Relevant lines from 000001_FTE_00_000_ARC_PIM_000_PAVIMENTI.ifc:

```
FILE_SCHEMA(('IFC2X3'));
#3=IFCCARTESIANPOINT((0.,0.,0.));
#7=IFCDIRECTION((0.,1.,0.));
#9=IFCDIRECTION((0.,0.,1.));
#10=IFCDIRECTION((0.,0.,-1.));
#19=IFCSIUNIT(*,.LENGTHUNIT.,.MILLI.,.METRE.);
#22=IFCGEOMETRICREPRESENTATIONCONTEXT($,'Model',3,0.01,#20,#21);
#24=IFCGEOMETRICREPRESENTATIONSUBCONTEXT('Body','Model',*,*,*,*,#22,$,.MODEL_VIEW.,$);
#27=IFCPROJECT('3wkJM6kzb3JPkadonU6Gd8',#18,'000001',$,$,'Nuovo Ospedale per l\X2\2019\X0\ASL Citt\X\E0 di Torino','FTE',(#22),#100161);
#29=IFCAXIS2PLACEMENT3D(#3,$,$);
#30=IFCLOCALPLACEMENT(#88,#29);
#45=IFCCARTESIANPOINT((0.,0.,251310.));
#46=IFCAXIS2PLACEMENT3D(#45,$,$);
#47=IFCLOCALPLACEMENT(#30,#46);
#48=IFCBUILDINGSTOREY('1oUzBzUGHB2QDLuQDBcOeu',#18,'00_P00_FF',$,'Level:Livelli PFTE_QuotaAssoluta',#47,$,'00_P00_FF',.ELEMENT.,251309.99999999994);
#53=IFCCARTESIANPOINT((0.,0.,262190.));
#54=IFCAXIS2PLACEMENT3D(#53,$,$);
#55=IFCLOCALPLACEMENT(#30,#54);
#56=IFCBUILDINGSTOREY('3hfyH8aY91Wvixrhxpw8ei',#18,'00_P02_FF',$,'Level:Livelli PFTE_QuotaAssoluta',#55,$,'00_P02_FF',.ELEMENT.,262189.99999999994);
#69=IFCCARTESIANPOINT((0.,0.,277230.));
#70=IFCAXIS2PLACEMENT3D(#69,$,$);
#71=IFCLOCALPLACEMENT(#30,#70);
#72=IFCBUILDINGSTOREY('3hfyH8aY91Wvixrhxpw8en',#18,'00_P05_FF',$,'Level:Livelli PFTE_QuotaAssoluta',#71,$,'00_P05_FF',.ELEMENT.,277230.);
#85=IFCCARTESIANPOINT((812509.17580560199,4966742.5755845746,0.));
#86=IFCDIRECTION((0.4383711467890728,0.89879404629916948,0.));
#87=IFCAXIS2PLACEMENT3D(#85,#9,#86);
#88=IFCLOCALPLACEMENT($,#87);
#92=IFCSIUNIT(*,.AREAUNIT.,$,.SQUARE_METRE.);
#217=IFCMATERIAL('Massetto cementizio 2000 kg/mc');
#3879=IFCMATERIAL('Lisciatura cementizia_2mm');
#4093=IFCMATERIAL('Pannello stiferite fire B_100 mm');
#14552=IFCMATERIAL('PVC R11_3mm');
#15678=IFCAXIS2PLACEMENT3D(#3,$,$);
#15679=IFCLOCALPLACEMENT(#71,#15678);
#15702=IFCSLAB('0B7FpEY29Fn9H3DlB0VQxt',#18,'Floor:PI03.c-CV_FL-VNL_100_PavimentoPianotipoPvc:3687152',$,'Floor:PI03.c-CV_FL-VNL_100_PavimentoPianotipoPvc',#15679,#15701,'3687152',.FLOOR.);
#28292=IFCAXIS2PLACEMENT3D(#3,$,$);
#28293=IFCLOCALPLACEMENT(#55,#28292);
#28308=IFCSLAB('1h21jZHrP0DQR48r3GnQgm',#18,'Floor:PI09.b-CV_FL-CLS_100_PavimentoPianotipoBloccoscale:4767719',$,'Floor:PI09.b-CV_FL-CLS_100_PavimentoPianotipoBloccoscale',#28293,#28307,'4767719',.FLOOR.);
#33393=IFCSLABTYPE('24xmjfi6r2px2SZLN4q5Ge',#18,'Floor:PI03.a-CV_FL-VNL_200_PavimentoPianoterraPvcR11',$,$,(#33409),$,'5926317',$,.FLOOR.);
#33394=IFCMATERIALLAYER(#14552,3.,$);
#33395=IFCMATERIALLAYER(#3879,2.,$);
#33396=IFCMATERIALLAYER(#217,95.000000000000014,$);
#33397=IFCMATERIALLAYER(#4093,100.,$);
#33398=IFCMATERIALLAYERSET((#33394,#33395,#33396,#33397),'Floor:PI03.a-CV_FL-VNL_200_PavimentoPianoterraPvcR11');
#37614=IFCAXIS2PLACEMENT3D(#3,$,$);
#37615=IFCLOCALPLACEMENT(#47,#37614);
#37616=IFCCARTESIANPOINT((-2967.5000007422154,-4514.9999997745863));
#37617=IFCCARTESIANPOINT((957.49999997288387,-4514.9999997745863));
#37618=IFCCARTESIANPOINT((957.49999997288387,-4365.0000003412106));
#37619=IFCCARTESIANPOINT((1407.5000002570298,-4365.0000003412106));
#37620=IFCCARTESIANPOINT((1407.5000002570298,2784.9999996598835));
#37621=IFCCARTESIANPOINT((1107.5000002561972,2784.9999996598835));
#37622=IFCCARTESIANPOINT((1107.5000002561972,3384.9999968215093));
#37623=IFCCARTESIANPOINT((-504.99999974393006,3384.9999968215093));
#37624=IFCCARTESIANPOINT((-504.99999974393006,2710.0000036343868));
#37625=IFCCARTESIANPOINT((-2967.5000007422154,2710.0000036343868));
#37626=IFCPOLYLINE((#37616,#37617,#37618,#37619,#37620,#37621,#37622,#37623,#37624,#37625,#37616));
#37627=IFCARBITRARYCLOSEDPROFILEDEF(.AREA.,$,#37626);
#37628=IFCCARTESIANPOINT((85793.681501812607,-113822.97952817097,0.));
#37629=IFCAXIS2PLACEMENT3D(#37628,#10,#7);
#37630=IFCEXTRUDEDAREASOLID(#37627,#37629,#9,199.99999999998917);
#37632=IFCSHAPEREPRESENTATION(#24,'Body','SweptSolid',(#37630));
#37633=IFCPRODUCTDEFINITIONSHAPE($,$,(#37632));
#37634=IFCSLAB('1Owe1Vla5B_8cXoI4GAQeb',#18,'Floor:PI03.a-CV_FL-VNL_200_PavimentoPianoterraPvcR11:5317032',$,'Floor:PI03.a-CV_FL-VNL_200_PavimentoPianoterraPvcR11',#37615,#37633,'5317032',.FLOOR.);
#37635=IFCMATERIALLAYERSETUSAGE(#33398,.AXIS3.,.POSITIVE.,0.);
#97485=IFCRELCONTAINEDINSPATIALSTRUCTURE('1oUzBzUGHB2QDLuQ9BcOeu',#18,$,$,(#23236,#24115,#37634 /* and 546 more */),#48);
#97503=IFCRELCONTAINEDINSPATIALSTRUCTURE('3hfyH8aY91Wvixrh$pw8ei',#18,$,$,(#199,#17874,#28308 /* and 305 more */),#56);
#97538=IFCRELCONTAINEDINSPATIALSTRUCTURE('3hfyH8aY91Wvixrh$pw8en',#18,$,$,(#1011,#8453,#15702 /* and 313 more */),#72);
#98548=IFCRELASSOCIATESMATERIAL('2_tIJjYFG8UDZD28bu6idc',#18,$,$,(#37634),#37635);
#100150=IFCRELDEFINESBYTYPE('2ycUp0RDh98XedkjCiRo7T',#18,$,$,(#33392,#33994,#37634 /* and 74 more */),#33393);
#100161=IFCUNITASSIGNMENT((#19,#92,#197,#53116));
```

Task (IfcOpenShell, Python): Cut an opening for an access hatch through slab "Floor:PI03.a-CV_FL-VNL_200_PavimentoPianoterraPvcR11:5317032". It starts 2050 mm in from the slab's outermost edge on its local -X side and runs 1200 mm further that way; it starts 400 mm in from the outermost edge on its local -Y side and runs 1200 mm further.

```python
import numpy as np
import ifcopenshell
import ifcopenshell.api.feature
import ifcopenshell.api.geometry
import ifcopenshell.api.root
import ifcopenshell.geom
import ifcopenshell.util.placement
import ifcopenshell.util.representation
import ifcopenshell.util.shape
import ifcopenshell.util.unit

model = ifcopenshell.open("000001_FTE_00_000_ARC_PIM_000_PAVIMENTI.ifc")
unit_scale = ifcopenshell.util.unit.calculate_unit_scale(model)
settings = ifcopenshell.geom.settings()


def volume(element):
    """Net volume in cubic metres, openings subtracted."""
    shape = ifcopenshell.geom.create_shape(settings, element)
    return ifcopenshell.util.shape.get_volume(shape.geometry)


slab = model.by_id(37634)
before = volume(slab)

# Extent in the slab's own axes, in metres. The edges named are its -X and -Y sides.
slab_shape = ifcopenshell.geom.create_shape(settings, slab)
vertices = ifcopenshell.util.shape.get_vertices(slab_shape.geometry)
x_min, y_min, bottom = vertices.min(axis=0)
top = vertices[:, 2].max()

opening = ifcopenshell.api.root.create_entity(model, ifc_class="IfcOpeningElement", name="Access hatch opening")
context = ifcopenshell.util.representation.get_context(model, "Model", "Body", "MODEL_VIEW")
width, depth = 1.2, 1.2
outline = [(0.0, 0.0), (width, 0.0), (width, depth), (0.0, depth), (0.0, 0.0)]
# Overshoot both faces by 50 mm so the cut is clean.
shape = ifcopenshell.api.geometry.add_slab_representation(
    model, context=context, depth=top - bottom + 0.1, polyline=outline
)
ifcopenshell.api.geometry.assign_representation(model, product=opening, representation=shape)

matrix = ifcopenshell.util.placement.get_local_placement(slab.ObjectPlacement)
matrix[:, 3] = matrix @ np.append(np.array([x_min + 2.05, y_min + 0.4, bottom - 0.05]) / unit_scale, 1.0)
ifcopenshell.api.geometry.edit_object_placement(model, product=opening, matrix=matrix, is_si=False)
ifcopenshell.api.feature.add_feature(model, feature=opening, element=slab)

after = volume(slab)

print(f"slab volume {before:.3f} -> {after:.3f} m3")

model.write("000001_FTE_00_000_ARC_PIM_000_PAVIMENTI_edited.ifc")
```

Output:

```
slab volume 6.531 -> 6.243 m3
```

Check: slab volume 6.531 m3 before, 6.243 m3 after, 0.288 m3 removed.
